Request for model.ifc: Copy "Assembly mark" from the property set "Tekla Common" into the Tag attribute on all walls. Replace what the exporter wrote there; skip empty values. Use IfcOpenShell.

First a look at what the model holds.

```python
import ifcopenshell
import ifcopenshell.util.element

model = ifcopenshell.open("model.ifc")
print(model.schema)
walls = model.by_type("IfcWall")
print(len(walls), "walls")
for e in walls[:8]:
    source = ifcopenshell.util.element.get_pset(e, "Tekla Common", "Assembly mark")
    target = e.Tag
    print(e.id(), repr(source), repr(target), sep=" | ")
```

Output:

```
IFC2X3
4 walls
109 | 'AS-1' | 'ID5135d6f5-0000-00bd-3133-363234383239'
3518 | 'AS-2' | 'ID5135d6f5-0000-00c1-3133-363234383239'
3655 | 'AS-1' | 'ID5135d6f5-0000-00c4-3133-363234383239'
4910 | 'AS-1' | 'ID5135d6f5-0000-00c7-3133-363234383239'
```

```python
import ifcopenshell
import ifcopenshell.util.element

model = ifcopenshell.open("model.ifc")

count = 0
for e in model.by_type("IfcWall"):
    value = ifcopenshell.util.element.get_pset(e, "Tekla Common", "Assembly mark")
    current = e.Tag
    if not value or not value.strip() or current == value:
        continue
    e.Tag = value
    count += 1

print(count, "walls updated")

model.write("model_v2.ifc")
```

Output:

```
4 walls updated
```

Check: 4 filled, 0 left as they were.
